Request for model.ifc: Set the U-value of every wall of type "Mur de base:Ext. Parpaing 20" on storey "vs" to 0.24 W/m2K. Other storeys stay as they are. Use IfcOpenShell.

First a look at what the model holds.

```python
import ifcopenshell
import ifcopenshell.util.element

model = ifcopenshell.open("model.ifc")
print(model.schema)
storey = next(s for s in model.by_type("IfcBuildingStorey") if s.Name == "vs")
walls = [e for e in ifcopenshell.util.element.get_decomposition(storey) if e.is_a("IfcWall")]
seen = {}
for e in walls:
    element_type = ifcopenshell.util.element.get_type(e)
    key = (element_type.Name if element_type != e and element_type else None, ifcopenshell.util.element.get_pset(e, "Pset_WallCommon", "ThermalTransmittance"))
    seen[key] = seen.get(key, 0) + 1
for (name, value), count in sorted(seen.items(), key=str):
    print(count, "x", name, "|", value)
```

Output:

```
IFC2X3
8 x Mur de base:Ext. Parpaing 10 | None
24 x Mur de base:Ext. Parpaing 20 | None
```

```python
import ifcopenshell
import ifcopenshell.api.pset
import ifcopenshell.util.element

model = ifcopenshell.open("model.ifc")

storey = next(s for s in model.by_type("IfcBuildingStorey") if s.Name == "vs")
walls = [e for e in ifcopenshell.util.element.get_decomposition(storey) if e.is_a("IfcWall")]

count = 0
for e in walls:
    element_type = ifcopenshell.util.element.get_type(e)
    if element_type in (None, e) or element_type.Name != "Mur de base:Ext. Parpaing 20":
        continue
    # add_pset returns the element's existing set when there is one.
    pset = ifcopenshell.api.pset.add_pset(model, product=e, name="Pset_WallCommon")
    ifcopenshell.api.pset.edit_pset(model, pset=pset, properties={"ThermalTransmittance": 0.24})
    count += 1

print(count, "walls updated")

model.write("model_v2.ifc")
```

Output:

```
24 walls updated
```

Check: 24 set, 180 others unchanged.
